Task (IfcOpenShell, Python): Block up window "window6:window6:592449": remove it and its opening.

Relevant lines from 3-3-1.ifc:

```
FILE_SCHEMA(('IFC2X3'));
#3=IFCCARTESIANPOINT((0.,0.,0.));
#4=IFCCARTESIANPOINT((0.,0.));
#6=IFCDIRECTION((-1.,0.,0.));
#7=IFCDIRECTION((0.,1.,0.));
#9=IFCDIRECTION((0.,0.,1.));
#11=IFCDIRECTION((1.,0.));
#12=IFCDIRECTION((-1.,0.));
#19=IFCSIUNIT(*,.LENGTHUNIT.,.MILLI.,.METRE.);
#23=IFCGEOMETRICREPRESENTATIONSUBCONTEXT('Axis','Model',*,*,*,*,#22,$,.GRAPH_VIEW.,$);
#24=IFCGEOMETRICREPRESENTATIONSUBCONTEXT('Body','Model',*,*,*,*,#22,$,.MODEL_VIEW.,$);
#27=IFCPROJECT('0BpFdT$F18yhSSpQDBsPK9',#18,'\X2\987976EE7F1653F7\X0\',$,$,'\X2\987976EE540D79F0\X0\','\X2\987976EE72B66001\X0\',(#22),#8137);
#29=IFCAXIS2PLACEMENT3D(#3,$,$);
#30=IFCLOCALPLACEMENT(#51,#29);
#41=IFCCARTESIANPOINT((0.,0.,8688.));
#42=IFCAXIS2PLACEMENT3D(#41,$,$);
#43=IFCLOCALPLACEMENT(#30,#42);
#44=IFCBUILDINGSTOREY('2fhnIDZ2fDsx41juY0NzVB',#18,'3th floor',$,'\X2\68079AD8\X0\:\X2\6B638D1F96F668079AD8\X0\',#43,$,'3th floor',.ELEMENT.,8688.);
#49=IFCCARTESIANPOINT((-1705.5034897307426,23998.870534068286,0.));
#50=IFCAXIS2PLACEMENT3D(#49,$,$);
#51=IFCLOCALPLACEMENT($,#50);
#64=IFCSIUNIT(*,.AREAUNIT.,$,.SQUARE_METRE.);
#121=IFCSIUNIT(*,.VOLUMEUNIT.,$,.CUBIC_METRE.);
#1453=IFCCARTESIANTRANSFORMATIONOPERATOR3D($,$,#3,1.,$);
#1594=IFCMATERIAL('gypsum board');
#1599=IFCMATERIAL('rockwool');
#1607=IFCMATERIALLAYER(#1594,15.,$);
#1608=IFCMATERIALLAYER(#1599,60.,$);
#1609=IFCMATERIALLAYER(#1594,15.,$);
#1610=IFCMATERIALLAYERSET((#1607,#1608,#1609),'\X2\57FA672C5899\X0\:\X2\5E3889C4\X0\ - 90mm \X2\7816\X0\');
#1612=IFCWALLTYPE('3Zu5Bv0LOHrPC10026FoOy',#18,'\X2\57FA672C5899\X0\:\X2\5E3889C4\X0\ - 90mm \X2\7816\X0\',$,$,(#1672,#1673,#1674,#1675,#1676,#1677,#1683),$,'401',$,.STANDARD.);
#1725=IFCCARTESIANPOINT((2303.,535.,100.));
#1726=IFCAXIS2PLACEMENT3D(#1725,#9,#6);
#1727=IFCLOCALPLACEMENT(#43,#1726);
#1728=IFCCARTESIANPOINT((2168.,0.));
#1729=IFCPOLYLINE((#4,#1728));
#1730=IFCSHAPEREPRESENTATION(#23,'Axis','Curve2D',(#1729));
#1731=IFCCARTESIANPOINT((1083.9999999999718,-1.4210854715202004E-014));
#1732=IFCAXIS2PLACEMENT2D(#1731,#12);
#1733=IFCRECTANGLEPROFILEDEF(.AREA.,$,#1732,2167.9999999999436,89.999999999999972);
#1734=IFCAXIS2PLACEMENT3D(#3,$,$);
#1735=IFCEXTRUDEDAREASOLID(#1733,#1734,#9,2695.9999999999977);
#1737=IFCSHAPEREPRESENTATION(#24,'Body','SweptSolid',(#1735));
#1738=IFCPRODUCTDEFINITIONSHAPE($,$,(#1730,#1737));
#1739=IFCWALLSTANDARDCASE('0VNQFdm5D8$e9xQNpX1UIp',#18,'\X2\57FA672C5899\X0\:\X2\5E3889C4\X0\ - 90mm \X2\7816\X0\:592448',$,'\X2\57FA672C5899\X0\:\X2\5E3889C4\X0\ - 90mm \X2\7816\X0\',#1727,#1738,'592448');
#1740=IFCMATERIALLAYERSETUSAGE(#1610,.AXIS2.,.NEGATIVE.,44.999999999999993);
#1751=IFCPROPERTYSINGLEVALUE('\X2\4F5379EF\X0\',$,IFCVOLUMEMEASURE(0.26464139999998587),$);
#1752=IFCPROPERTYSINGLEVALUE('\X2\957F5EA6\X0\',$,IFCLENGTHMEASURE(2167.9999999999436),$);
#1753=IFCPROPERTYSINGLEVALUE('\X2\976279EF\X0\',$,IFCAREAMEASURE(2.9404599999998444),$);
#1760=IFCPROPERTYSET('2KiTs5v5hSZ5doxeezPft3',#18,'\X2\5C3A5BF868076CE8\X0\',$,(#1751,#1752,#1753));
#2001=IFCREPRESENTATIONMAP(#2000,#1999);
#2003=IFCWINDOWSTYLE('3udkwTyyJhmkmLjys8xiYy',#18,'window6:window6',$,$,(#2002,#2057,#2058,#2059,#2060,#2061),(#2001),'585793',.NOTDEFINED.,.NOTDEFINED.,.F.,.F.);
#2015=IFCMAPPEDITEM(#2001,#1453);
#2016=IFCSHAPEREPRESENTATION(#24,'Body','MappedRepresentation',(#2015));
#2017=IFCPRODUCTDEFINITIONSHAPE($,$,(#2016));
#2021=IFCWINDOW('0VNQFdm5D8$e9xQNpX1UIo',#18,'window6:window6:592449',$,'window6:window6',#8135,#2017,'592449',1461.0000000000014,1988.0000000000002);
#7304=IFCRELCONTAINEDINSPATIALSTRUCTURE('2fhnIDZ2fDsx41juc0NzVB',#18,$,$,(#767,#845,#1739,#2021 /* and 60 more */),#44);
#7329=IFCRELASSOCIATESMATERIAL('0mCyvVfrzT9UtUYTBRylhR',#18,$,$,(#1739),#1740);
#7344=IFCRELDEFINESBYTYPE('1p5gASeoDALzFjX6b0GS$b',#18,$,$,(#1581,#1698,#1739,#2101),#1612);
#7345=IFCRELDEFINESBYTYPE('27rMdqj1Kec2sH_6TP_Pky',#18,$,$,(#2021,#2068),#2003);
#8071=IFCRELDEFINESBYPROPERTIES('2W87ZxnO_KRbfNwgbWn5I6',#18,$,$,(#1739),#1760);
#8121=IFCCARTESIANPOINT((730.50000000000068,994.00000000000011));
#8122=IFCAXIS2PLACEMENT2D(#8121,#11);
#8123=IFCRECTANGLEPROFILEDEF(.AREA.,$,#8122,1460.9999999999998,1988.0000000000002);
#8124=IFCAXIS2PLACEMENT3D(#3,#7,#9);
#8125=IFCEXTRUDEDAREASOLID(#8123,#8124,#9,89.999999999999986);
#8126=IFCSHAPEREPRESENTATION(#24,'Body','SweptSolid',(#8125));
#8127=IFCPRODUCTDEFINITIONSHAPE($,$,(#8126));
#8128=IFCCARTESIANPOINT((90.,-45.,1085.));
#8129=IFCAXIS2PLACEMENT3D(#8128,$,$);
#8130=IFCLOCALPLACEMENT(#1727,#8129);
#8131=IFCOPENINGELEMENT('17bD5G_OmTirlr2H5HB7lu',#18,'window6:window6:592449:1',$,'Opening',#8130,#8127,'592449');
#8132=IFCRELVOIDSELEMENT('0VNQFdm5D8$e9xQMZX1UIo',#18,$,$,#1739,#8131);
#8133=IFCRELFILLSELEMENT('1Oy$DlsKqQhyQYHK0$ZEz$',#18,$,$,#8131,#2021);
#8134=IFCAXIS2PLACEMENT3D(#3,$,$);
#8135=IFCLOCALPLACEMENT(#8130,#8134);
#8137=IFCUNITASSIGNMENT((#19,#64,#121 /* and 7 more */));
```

```python
import ifcopenshell
import ifcopenshell.api.feature
import ifcopenshell.api.pset
import ifcopenshell.api.root
import ifcopenshell.geom
import ifcopenshell.util.element
import ifcopenshell.util.shape
import ifcopenshell.util.unit

model = ifcopenshell.open("3-3-1.ifc")
area_scale = ifcopenshell.util.unit.calculate_unit_scale(model, "AREAUNIT")
volume_scale = ifcopenshell.util.unit.calculate_unit_scale(model, "VOLUMEUNIT")
settings = ifcopenshell.geom.settings()


def volume(element):
    """Net volume in cubic metres, openings subtracted."""
    shape = ifcopenshell.geom.create_shape(settings, element)
    return ifcopenshell.util.shape.get_volume(shape.geometry)


window = model.by_id(2021)
opening = window.FillsVoids[0].RelatingOpeningElement
wall = opening.VoidsElements[0].RelatingBuildingElement
before = volume(wall)

ifcopenshell.api.root.remove_product(model, product=window)
ifcopenshell.api.feature.remove_feature(model, feature=opening)

after = volume(wall)
thickness = 0.09  # wall thickness in metres

# Update the wall's stored quantities.
pset = model.by_id(ifcopenshell.util.element.get_pset(wall, "尺寸标注", should_inherit=False)["id"])
ifcopenshell.api.pset.edit_pset(model, pset=pset, properties={
    "体积": model.create_entity("IfcVolumeMeasure", after / volume_scale),
    "面积": model.create_entity("IfcAreaMeasure", after / thickness / area_scale),
})

print(f"wall volume {before:.3f} -> {after:.3f} m3")

model.write("3-3-1_edited.ifc")
```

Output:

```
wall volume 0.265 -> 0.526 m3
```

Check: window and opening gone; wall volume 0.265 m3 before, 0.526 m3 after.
